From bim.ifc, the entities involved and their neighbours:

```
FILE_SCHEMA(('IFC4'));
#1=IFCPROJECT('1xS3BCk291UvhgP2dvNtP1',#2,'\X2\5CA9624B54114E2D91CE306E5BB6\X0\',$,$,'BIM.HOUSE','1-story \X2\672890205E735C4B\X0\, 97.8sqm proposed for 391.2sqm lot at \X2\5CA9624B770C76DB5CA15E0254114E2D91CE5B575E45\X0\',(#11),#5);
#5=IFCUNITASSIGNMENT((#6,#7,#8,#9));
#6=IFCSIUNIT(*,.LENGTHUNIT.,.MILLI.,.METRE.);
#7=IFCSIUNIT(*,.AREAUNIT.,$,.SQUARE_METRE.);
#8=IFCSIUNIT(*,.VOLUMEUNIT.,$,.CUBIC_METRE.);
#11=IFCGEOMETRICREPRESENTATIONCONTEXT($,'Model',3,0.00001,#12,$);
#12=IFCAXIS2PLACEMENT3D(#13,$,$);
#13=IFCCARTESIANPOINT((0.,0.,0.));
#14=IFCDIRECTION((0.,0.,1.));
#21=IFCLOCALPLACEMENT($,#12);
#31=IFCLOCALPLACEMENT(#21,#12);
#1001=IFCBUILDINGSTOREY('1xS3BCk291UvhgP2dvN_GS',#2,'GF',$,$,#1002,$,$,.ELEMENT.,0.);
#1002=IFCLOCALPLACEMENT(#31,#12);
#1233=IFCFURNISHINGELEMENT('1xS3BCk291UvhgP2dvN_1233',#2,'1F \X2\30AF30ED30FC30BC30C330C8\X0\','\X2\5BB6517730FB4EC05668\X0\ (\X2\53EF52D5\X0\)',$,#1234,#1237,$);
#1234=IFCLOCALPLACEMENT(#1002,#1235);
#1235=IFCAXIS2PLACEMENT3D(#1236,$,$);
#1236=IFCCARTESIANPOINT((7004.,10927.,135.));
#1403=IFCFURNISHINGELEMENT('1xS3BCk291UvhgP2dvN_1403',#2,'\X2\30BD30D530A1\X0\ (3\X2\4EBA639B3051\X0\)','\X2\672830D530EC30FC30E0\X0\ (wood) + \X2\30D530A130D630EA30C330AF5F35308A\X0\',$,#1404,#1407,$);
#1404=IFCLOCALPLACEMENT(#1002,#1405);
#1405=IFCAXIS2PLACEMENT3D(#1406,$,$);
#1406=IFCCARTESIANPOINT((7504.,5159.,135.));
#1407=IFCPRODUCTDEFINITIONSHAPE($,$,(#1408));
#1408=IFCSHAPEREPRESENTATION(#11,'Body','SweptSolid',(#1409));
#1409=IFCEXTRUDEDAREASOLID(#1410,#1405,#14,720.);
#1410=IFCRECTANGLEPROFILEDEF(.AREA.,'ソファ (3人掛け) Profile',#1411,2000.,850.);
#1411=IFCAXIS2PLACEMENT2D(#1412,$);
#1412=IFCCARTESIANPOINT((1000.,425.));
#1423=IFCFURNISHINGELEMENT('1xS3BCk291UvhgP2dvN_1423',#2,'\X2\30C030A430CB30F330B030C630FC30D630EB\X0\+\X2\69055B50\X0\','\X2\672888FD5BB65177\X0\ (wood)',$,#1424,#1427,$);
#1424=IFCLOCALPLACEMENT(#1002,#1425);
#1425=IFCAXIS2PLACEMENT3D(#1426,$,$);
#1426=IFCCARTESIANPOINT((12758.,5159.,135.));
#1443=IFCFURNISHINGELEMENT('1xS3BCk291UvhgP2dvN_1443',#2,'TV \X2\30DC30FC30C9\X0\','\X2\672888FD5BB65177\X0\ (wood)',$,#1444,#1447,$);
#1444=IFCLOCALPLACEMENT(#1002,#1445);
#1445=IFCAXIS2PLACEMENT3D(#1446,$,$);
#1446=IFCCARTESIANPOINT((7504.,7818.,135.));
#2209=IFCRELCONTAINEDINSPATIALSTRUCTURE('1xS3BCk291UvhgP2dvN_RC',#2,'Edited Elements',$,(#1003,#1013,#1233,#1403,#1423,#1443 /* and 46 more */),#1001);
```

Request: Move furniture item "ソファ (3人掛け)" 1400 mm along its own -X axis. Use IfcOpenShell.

```python
import ifcopenshell
import ifcopenshell.api.geometry
import ifcopenshell.util.placement
import ifcopenshell.util.unit

model = ifcopenshell.open("bim.ifc")
unit_scale = ifcopenshell.util.unit.calculate_unit_scale(model)

item = model.by_guid("1xS3BCk291UvhgP2dvN_1403")
matrix = ifcopenshell.util.placement.get_local_placement(item.ObjectPlacement)
matrix[:3, 3] -= matrix[:3, 0] * 1.4 / unit_scale
ifcopenshell.api.geometry.edit_object_placement(model, product=item, matrix=matrix, is_si=False)

print(ifcopenshell.util.placement.get_local_placement(item.ObjectPlacement).round(3) + 0.0)

model.write("bim_edited.ifc")
```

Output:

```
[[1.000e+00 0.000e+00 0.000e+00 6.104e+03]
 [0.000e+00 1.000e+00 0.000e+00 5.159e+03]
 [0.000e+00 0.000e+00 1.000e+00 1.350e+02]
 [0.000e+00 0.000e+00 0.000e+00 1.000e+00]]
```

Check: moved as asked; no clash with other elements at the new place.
